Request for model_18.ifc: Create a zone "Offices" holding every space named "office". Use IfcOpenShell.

First a look at what the model holds.

```python
import ifcopenshell

model = ifcopenshell.open("model_18.ifc")
print(model.schema)
seen = {}
for space in model.by_type("IfcSpace"):
    seen[space.LongName] = seen.get(space.LongName, 0) + 1
for name, count in sorted(seen.items(), key=str):
    print(count, "x", name)
print("zones:", [z.Name for z in model.by_type("IfcZone")][:20])
```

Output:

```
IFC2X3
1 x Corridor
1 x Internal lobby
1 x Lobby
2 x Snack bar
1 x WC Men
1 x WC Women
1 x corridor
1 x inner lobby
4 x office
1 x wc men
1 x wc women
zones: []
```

```python
import ifcopenshell
import ifcopenshell.api.group
import ifcopenshell.api.root

model = ifcopenshell.open("model_18.ifc")

names = {"office"}
spaces = [s for s in model.by_type("IfcSpace") if s.LongName in names]

zone = ifcopenshell.api.root.create_entity(model, ifc_class="IfcZone", name="Offices")
ifcopenshell.api.group.assign_group(model, products=spaces, group=zone)
print(len(spaces), "spaces in", zone.Name)

model.write("model_18-out.ifc")
```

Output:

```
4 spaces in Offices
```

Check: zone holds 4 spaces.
